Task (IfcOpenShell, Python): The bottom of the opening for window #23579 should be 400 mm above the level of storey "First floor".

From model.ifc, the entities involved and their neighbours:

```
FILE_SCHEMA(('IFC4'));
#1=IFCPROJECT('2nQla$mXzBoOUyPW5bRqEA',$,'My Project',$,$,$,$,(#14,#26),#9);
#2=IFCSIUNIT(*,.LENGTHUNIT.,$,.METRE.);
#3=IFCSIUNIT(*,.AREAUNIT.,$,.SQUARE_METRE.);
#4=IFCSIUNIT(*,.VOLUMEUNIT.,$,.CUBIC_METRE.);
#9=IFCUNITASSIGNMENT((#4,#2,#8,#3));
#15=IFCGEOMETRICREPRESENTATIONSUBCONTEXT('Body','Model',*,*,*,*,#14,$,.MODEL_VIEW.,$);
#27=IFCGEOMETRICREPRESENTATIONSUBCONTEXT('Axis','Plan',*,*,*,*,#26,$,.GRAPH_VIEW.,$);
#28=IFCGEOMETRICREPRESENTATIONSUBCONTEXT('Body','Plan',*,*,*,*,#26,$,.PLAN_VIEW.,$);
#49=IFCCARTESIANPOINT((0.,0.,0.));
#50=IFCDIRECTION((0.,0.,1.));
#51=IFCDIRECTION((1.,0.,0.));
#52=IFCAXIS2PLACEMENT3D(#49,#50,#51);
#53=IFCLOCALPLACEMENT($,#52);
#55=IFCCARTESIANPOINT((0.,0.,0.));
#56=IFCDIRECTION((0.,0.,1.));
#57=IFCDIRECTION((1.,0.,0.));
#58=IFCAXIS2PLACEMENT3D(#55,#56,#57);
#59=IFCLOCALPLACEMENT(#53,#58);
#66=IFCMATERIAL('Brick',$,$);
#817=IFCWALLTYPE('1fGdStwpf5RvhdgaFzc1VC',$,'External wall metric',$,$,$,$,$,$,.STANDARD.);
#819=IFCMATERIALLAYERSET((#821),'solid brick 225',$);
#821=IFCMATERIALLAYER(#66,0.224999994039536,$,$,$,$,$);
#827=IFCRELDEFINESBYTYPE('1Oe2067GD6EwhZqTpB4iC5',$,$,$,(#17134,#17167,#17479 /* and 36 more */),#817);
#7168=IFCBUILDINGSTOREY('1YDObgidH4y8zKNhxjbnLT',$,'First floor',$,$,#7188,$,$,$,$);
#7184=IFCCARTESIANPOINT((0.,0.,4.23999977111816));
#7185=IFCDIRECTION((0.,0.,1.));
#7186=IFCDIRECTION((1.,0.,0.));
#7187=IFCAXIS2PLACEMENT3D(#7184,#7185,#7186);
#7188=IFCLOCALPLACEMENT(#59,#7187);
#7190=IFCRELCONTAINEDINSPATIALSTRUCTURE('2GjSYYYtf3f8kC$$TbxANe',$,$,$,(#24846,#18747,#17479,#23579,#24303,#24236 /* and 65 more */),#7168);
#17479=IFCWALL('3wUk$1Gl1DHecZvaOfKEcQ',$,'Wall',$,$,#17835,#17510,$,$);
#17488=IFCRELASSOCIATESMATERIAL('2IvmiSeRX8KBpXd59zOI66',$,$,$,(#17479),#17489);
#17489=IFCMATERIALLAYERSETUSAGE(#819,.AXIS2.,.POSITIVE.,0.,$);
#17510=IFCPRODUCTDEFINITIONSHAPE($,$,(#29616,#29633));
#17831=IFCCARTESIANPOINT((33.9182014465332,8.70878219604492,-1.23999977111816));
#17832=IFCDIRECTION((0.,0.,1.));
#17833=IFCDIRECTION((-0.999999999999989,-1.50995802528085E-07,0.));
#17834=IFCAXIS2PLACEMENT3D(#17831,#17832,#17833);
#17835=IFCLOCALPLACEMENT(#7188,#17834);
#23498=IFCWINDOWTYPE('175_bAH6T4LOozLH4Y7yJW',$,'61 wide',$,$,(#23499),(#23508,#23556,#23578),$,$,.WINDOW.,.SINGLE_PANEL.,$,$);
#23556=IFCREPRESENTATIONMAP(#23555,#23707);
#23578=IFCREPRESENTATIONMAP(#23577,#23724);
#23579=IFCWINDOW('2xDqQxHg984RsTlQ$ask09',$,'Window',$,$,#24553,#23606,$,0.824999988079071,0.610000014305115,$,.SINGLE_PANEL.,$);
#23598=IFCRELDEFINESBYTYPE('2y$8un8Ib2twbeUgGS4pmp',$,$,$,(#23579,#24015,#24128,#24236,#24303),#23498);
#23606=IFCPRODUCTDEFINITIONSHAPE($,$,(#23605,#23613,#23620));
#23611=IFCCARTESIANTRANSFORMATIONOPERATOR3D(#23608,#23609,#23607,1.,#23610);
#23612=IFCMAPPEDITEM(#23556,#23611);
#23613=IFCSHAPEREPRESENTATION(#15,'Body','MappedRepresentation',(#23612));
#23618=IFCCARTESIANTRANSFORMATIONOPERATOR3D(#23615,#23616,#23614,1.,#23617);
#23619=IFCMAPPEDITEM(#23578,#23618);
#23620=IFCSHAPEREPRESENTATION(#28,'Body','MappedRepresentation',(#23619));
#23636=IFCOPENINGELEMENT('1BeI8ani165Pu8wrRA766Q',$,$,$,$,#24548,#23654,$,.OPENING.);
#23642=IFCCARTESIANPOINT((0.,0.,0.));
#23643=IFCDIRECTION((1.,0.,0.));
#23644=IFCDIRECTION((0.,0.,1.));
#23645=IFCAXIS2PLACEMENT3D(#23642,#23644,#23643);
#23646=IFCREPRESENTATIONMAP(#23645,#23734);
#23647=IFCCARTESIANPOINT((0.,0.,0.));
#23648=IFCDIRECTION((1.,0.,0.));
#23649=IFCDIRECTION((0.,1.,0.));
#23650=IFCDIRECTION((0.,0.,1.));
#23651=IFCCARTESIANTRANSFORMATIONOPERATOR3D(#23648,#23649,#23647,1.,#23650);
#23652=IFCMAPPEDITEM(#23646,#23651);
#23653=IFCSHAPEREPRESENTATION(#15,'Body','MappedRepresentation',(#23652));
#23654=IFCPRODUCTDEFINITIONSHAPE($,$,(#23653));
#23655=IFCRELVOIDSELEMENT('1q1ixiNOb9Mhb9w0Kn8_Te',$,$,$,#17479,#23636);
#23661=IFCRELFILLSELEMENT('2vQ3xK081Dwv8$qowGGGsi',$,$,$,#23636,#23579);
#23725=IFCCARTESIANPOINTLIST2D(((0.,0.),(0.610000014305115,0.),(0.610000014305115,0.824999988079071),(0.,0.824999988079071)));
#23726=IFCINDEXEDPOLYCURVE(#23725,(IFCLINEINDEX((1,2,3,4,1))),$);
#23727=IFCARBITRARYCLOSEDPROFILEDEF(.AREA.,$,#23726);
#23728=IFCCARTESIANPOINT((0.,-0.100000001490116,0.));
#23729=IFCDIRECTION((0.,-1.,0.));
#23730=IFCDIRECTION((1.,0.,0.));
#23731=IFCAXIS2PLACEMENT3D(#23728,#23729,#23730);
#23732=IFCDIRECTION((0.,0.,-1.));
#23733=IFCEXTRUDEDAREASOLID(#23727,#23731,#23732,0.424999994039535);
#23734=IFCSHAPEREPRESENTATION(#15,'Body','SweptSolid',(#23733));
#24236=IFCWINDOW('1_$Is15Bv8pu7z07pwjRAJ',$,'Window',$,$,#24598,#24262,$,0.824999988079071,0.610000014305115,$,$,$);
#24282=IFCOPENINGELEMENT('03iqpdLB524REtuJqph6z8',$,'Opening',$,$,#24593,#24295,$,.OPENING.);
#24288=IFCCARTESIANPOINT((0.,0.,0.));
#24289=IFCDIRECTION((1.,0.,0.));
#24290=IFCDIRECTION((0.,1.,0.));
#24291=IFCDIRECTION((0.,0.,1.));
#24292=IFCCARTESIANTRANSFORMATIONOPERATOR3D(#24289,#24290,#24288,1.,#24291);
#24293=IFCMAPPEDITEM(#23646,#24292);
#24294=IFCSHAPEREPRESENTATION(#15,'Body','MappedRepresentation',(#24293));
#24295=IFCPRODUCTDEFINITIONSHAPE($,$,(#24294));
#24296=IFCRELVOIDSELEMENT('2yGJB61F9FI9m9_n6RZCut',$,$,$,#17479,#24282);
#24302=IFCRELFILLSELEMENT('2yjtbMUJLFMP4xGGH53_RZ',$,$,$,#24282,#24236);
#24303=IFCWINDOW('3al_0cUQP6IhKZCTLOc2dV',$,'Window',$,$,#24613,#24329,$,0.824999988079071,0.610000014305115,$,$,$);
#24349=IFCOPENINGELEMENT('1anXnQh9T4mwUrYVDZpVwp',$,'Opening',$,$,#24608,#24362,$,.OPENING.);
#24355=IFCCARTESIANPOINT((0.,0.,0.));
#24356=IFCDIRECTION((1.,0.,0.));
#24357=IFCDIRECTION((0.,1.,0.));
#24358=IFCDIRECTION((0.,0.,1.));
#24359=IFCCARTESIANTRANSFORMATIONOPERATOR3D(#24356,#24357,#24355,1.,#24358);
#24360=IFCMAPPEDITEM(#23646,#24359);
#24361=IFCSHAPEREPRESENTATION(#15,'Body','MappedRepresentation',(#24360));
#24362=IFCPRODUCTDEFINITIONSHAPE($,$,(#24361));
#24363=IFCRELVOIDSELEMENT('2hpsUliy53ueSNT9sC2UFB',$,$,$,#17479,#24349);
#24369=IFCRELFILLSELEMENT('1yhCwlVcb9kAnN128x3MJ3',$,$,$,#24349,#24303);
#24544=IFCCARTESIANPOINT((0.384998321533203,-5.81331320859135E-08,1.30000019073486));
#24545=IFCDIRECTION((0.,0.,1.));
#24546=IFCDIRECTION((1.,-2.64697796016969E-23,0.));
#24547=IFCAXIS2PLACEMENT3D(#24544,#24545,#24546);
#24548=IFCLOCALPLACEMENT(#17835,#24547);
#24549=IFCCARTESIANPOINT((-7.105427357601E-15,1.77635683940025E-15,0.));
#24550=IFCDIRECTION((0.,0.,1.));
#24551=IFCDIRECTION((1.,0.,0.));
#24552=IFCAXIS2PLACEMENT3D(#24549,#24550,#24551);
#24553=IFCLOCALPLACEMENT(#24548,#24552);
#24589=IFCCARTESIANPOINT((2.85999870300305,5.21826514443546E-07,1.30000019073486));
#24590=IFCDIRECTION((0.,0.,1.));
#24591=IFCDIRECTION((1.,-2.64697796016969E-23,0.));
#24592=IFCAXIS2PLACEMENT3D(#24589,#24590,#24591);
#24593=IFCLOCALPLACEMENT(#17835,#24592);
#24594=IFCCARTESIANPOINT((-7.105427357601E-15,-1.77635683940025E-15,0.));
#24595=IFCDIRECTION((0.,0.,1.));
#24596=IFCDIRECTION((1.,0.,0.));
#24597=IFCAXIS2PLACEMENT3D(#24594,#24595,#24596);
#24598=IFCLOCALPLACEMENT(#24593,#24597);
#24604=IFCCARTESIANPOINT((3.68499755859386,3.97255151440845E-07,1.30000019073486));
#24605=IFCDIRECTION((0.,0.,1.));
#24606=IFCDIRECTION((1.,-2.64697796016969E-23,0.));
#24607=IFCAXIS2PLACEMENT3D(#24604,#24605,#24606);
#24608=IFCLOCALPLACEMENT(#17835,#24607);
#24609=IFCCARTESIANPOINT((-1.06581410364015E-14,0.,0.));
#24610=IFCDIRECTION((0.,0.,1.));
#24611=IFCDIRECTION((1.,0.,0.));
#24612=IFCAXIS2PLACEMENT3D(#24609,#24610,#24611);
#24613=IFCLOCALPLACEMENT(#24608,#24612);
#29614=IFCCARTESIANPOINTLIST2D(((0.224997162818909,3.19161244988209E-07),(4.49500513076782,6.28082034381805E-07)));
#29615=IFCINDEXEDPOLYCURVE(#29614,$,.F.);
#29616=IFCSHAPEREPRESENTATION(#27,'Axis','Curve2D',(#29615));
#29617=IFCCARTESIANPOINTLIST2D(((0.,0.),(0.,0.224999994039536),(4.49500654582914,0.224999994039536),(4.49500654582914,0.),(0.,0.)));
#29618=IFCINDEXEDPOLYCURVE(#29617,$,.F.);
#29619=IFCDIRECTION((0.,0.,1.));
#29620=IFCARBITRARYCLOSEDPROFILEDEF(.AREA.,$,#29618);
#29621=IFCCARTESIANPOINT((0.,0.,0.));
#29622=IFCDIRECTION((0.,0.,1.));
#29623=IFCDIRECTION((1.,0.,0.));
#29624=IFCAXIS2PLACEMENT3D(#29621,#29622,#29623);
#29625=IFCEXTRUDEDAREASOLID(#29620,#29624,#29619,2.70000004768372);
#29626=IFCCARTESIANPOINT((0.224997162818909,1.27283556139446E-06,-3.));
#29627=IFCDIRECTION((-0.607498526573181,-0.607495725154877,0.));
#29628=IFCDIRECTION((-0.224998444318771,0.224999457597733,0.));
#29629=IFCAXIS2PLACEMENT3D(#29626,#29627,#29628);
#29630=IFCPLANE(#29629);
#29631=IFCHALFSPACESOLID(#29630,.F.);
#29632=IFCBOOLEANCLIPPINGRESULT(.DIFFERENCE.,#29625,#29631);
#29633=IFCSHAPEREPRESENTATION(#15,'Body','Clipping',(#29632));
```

```python
import numpy as np
import ifcopenshell
import ifcopenshell.api.geometry
import ifcopenshell.geom
import ifcopenshell.util.element
import ifcopenshell.util.placement
import ifcopenshell.util.shape
import ifcopenshell.util.unit

model = ifcopenshell.open("model.ifc")
unit_scale = ifcopenshell.util.unit.calculate_unit_scale(model)

window = model.by_id(23579)
opening = window.FillsVoids[0].RelatingOpeningElement
storey = ifcopenshell.util.element.get_container(window, ifc_class="IfcBuildingStorey")
level = ifcopenshell.util.placement.get_local_placement(storey.ObjectPlacement)[2, 3]

# The opening's origin need not be at the sill, so measure its lowest point.
shape = ifcopenshell.geom.create_shape(ifcopenshell.geom.settings(), opening)
bottom = ifcopenshell.util.shape.get_shape_bottom_elevation(shape, shape.geometry) / unit_scale
dz = level + 0.4 / unit_scale - bottom

shift = np.array([0.0, 0.0, dz])
# The window is placed relative to its opening, so it follows when the opening moves.
matrix = ifcopenshell.util.placement.get_local_placement(opening.ObjectPlacement)
matrix[:3, 3] += shift
ifcopenshell.api.geometry.edit_object_placement(
    model, product=opening, matrix=matrix, is_si=False, should_transform_children=True
)

print(f"moved by {dz * unit_scale:+.3f} m")

model.write("model_edited.ifc")
```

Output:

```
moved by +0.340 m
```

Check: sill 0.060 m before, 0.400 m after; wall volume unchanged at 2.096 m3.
